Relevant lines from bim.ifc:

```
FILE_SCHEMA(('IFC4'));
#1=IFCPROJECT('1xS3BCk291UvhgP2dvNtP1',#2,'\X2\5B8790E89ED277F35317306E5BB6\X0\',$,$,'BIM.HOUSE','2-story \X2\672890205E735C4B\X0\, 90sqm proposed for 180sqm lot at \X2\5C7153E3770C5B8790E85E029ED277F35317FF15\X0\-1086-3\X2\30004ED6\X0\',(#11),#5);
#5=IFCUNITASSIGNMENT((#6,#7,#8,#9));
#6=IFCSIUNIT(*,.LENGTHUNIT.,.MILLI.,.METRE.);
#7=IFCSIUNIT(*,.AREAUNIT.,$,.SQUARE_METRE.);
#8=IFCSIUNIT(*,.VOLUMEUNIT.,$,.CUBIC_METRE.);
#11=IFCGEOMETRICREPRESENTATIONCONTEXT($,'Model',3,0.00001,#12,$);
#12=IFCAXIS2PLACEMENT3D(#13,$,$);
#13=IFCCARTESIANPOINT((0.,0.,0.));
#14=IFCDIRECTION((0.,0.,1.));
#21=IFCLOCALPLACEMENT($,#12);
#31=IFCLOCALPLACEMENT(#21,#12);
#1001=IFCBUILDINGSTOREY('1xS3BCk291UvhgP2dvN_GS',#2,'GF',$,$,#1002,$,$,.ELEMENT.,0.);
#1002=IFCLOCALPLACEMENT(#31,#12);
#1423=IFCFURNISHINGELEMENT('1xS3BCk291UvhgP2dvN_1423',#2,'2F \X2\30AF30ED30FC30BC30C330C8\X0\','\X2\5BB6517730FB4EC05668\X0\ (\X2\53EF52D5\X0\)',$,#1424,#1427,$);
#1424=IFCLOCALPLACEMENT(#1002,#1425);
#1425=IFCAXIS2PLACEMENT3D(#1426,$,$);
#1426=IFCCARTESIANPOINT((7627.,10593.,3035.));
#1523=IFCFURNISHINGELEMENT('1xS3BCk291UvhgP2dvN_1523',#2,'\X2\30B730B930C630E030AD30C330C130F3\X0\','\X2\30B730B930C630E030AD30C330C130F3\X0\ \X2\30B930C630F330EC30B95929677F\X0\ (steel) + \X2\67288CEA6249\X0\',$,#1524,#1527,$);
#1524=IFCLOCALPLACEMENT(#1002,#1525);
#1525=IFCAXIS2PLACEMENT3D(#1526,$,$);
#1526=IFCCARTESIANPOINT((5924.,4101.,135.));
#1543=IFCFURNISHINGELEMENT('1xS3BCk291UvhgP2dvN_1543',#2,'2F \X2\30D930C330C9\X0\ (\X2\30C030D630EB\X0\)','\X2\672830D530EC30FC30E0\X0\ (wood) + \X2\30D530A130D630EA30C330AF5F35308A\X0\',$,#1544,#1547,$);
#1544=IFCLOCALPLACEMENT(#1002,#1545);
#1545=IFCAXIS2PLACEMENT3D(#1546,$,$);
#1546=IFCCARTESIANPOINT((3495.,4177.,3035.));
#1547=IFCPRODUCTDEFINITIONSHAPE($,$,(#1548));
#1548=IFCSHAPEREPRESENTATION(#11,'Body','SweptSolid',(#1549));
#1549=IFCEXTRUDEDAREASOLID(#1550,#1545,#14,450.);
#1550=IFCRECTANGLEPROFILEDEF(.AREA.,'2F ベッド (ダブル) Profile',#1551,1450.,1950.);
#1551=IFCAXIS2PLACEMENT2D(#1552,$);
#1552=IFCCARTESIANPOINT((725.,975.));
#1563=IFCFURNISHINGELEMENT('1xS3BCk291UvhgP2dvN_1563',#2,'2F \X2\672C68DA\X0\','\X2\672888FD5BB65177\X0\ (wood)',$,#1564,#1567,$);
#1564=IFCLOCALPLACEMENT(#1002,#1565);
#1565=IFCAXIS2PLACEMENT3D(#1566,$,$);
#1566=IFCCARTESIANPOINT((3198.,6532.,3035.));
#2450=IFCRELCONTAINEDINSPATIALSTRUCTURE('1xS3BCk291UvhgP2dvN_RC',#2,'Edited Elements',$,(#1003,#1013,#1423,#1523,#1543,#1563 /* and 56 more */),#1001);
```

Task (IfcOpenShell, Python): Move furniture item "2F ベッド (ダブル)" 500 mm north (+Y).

```python
import ifcopenshell
import ifcopenshell.api.geometry
import ifcopenshell.util.placement

model = ifcopenshell.open("bim.ifc")

item = model.by_id(1543)
matrix = ifcopenshell.util.placement.get_local_placement(item.ObjectPlacement)
matrix[1, 3] += 500.0
ifcopenshell.api.geometry.edit_object_placement(model, product=item, matrix=matrix, is_si=False)

print(ifcopenshell.util.placement.get_local_placement(item.ObjectPlacement).round(3) + 0.0)

model.write("bim-out.ifc")
```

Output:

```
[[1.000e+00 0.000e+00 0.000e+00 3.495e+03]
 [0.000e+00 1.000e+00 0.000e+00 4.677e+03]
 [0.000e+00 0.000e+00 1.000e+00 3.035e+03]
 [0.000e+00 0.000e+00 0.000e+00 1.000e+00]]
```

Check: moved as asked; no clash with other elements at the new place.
